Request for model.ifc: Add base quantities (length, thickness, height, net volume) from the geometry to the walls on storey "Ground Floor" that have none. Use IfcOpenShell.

First a look at what the model holds.

```python
import ifcopenshell
import ifcopenshell.util.element
import ifcopenshell.util.unit

model = ifcopenshell.open("model.ifc")
print(model.schema)
for unit_type in ("LENGTHUNIT", "AREAUNIT", "VOLUMEUNIT"):
    print(unit_type, ifcopenshell.util.unit.calculate_unit_scale(model, unit_type))
storey = next(s for s in model.by_type("IfcBuildingStorey") if s.Name == "Ground Floor")
walls = [e for e in ifcopenshell.util.element.get_decomposition(storey) if e.is_a("IfcWall")]
for e in sorted(walls, key=lambda e: e.id()):
    print(e.id(), e.is_a(), e.Name, list(ifcopenshell.util.element.get_psets(e, qtos_only=True)), sep=" | ")
```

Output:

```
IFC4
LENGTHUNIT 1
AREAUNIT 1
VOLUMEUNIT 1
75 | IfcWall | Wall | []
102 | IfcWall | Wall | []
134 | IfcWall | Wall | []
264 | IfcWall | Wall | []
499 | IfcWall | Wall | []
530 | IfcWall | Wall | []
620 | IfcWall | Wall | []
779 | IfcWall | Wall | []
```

```python
import ifcopenshell
import ifcopenshell.api.pset
import ifcopenshell.geom
import ifcopenshell.util.element
import ifcopenshell.util.shape
import ifcopenshell.util.unit

model = ifcopenshell.open("model.ifc")
unit_scale = ifcopenshell.util.unit.calculate_unit_scale(model)
volume_scale = ifcopenshell.util.unit.calculate_unit_scale(model, "VOLUMEUNIT")
settings = ifcopenshell.geom.settings()

storey = next(s for s in model.by_type("IfcBuildingStorey") if s.Name == "Ground Floor")
walls = [e for e in ifcopenshell.util.element.get_decomposition(storey) if e.is_a("IfcWall")]

for e in sorted(walls, key=lambda e: e.id()):
    if ifcopenshell.util.element.get_psets(e, qtos_only=True, should_inherit=False):
        continue
    # Geometry comes back in metres, in the element's own axes.
    shape = ifcopenshell.geom.create_shape(settings, e)
    values = {
        "Length": ifcopenshell.util.shape.get_x(shape.geometry) / unit_scale,
        "Width": ifcopenshell.util.shape.get_y(shape.geometry) / unit_scale,
        "Height": ifcopenshell.util.shape.get_z(shape.geometry) / unit_scale,
        "NetVolume": ifcopenshell.util.shape.get_volume(shape.geometry) / volume_scale,
    }
    qto = ifcopenshell.api.pset.add_qto(model, product=e, name="Qto_WallBaseQuantities")
    ifcopenshell.api.pset.edit_qto(model, qto=qto, properties=values)
    print(e.id(), {k: round(v, 3) for k, v in values.items()})

model.write("model_updated.ifc")
```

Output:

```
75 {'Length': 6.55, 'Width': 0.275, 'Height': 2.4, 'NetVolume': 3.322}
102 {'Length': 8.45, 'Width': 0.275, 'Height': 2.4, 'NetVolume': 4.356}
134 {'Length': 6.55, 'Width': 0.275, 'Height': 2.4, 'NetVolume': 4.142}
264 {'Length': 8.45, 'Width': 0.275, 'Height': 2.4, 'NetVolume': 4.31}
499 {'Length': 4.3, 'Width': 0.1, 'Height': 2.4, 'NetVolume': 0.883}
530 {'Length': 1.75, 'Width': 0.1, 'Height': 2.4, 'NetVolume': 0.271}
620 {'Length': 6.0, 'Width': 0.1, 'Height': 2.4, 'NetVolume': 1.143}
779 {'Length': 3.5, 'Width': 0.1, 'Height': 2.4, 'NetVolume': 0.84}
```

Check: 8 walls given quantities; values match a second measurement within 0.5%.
